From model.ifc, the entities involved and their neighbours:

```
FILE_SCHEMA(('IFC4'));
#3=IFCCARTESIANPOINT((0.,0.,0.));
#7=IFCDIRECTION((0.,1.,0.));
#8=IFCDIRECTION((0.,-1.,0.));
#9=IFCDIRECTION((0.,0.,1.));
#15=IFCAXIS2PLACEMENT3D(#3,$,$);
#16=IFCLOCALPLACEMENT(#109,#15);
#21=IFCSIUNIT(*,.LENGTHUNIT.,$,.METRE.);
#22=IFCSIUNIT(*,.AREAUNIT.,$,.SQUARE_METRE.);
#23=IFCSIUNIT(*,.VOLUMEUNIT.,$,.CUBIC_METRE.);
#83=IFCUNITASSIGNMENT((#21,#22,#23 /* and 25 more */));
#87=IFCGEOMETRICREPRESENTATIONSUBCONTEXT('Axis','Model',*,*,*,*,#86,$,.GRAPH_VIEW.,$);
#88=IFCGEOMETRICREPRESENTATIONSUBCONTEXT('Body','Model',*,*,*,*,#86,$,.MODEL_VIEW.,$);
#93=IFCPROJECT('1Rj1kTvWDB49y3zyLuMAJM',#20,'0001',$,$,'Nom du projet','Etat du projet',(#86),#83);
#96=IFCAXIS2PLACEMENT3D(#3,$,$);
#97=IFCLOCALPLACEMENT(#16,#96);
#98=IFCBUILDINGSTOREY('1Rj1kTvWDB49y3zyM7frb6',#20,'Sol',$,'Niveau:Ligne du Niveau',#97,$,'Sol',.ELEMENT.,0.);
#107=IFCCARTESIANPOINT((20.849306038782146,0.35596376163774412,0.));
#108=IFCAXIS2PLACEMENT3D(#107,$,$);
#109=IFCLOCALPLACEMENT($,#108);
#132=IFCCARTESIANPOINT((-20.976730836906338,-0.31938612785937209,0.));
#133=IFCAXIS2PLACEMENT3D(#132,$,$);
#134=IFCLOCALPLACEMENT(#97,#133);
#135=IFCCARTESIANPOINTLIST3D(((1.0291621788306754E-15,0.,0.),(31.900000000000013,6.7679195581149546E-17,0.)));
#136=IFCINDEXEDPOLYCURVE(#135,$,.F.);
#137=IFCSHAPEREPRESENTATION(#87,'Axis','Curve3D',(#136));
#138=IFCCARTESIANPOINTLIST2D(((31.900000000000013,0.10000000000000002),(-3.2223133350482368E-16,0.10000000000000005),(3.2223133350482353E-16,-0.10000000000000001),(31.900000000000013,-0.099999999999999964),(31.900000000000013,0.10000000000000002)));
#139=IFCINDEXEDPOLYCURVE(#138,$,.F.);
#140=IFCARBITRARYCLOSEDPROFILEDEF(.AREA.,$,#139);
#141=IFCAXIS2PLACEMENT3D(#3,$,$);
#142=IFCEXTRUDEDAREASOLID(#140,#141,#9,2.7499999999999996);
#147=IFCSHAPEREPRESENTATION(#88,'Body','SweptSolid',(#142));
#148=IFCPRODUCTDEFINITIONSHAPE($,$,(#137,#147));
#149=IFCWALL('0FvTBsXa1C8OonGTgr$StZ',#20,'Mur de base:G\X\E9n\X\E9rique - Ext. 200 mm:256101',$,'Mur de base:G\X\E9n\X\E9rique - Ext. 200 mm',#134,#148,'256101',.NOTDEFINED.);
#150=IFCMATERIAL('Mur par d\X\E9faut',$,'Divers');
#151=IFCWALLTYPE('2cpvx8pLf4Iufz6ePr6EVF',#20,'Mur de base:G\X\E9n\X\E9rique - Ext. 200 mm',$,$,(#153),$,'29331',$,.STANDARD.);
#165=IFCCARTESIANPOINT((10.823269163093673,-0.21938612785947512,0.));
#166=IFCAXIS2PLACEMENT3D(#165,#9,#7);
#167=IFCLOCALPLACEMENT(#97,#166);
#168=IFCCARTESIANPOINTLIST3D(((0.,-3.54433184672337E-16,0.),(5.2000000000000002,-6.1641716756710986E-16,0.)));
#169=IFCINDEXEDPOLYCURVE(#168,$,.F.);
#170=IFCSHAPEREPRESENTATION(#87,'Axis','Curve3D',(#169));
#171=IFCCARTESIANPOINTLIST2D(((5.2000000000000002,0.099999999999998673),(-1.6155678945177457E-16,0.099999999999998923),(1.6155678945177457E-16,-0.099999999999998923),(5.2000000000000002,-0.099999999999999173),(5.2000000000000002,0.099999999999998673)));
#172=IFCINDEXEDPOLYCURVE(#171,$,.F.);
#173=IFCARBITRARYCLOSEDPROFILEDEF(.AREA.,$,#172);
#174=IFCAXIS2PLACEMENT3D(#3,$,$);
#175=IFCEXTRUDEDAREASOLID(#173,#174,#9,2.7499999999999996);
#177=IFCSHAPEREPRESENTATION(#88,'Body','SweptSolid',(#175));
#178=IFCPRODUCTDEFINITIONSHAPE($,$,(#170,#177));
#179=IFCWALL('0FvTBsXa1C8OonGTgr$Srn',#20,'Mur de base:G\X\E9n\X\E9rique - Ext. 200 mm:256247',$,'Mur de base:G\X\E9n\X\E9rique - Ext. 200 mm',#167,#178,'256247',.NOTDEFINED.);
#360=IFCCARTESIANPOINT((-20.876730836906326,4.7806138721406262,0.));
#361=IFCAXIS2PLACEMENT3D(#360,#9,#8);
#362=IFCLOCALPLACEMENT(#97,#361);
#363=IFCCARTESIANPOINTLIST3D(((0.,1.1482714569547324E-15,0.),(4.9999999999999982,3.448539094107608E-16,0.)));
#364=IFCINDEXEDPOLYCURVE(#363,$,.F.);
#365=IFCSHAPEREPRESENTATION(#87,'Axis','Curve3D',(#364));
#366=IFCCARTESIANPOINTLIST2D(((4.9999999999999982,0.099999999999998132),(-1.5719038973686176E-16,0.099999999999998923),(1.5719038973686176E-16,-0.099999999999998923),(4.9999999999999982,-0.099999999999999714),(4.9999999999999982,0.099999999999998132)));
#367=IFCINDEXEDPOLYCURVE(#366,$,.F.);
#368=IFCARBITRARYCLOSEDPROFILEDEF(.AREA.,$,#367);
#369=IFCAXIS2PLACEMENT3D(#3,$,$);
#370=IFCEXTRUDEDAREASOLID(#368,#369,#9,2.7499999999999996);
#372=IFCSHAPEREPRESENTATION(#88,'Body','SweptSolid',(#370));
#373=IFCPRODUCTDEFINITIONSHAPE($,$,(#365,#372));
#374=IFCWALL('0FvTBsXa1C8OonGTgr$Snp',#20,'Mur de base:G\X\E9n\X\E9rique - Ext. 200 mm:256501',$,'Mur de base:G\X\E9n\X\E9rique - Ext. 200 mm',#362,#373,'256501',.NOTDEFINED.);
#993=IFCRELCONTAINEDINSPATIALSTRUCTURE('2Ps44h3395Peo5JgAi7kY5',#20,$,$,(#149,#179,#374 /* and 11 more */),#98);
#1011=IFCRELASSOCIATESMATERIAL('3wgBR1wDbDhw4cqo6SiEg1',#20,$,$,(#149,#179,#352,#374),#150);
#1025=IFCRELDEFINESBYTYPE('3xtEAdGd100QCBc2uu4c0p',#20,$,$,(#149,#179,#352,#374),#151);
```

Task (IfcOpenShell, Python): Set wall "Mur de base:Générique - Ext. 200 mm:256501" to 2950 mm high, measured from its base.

```python
import ifcopenshell
import ifcopenshell.geom
import ifcopenshell.util.representation
import ifcopenshell.util.shape
import ifcopenshell.util.unit

model = ifcopenshell.open("model.ifc")
unit_scale = ifcopenshell.util.unit.calculate_unit_scale(model)
settings = ifcopenshell.geom.settings()


def volume(element):
    """Net volume in cubic metres, openings subtracted."""
    shape = ifcopenshell.geom.create_shape(settings, element)
    return ifcopenshell.util.shape.get_volume(shape.geometry)


wall = model.by_id(374)
before = volume(wall)

body = ifcopenshell.util.representation.get_representation(wall, "Model", "Body")
solid = body.Items[0]
old_height = solid.Depth
solid.Depth = 2.95 / unit_scale
after = volume(wall)

print(f"height {old_height:g} -> {solid.Depth:g}, volume {before:.3f} -> {after:.3f} m3")

model.write("model_updated.ifc")
```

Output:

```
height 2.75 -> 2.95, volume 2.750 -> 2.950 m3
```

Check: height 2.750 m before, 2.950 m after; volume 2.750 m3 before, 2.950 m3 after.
